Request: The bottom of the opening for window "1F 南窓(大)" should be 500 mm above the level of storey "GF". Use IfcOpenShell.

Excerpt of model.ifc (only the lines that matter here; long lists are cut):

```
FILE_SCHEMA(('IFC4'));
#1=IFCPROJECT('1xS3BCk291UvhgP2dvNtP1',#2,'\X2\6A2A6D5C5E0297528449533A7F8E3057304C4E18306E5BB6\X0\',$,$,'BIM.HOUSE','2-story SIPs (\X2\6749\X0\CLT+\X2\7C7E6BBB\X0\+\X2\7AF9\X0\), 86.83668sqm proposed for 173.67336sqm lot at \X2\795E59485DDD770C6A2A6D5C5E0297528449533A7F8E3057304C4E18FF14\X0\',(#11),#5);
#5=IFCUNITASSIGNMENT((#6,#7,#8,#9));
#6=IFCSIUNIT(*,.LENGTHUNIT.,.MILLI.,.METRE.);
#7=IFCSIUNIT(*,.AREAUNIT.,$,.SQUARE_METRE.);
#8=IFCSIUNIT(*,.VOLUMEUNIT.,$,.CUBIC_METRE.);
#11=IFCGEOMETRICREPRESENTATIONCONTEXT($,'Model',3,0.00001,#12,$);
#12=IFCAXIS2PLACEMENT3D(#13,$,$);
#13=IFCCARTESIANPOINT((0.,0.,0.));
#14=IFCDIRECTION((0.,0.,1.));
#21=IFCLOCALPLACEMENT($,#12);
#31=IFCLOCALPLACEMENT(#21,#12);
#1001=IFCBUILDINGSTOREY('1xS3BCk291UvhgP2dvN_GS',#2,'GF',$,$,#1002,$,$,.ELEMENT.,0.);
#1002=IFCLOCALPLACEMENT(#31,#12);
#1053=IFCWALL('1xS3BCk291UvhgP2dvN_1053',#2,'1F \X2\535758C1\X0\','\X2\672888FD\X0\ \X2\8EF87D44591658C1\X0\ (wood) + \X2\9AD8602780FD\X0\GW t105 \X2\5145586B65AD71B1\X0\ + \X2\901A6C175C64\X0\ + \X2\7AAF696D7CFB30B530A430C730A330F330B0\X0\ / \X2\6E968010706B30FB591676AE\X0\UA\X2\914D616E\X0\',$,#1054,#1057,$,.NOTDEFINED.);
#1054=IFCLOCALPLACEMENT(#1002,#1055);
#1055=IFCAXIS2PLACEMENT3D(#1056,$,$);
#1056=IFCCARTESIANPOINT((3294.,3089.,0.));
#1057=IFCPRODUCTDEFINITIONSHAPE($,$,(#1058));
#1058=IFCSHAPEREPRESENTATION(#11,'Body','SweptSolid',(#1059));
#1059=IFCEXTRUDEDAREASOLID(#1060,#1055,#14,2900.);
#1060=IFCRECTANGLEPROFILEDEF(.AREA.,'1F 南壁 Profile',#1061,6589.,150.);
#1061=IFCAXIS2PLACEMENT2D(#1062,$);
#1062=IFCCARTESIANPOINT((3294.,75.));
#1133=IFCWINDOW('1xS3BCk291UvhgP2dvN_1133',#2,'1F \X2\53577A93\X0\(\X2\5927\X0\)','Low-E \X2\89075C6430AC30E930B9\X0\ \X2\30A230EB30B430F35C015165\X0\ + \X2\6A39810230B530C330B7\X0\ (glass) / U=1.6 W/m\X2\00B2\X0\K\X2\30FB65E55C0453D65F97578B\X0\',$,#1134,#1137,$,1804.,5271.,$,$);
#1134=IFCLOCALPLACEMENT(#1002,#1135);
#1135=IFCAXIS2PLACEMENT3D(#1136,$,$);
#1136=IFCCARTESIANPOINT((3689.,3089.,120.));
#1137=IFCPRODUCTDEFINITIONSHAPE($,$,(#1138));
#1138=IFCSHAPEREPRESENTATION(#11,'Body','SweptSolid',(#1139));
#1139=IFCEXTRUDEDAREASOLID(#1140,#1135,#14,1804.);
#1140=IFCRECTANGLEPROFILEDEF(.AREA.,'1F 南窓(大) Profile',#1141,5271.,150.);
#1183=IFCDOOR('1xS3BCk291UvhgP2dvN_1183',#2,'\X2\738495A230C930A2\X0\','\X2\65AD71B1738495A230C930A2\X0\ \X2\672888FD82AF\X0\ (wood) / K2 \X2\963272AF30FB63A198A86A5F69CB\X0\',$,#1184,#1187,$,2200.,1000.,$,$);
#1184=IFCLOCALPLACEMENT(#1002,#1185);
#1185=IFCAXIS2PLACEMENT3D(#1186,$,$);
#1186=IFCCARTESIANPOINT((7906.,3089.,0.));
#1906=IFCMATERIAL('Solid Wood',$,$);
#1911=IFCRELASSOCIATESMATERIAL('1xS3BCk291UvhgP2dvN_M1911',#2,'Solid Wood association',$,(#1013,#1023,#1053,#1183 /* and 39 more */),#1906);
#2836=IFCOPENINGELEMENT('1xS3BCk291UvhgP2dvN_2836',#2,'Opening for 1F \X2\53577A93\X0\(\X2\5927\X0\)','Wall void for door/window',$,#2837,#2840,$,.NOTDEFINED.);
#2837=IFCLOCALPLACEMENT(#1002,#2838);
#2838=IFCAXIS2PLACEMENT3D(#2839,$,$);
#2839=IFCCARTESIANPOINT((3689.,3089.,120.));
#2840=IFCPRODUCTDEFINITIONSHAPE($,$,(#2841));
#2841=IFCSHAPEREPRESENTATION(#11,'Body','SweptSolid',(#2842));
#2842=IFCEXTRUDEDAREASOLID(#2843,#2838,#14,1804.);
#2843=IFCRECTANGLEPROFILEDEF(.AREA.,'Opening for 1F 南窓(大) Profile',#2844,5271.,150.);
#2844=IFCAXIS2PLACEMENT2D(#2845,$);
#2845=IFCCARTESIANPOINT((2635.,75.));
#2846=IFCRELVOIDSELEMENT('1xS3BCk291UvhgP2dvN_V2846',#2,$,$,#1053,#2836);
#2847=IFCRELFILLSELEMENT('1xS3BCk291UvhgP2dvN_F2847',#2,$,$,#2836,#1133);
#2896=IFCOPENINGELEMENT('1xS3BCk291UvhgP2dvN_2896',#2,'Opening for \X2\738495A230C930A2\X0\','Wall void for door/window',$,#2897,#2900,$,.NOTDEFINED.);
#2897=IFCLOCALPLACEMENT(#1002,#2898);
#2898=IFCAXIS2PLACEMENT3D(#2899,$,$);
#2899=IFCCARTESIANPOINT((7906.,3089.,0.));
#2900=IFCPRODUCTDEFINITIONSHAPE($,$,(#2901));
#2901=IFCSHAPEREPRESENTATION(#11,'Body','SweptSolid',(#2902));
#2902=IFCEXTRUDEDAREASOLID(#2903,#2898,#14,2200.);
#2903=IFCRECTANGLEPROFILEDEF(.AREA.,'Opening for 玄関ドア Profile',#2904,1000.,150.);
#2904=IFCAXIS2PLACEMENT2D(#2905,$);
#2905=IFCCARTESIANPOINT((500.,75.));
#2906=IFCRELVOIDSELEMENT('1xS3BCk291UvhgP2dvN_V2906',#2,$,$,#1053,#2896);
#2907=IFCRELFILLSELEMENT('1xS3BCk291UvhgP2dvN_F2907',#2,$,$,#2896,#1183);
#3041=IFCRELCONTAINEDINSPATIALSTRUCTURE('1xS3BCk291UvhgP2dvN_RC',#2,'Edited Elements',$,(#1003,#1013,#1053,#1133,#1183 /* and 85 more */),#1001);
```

```python
import numpy as np
import ifcopenshell
import ifcopenshell.api.geometry
import ifcopenshell.geom
import ifcopenshell.util.element
import ifcopenshell.util.placement
import ifcopenshell.util.shape
import ifcopenshell.util.unit

model = ifcopenshell.open("model.ifc")
unit_scale = ifcopenshell.util.unit.calculate_unit_scale(model)

window = model.by_id(1133)
opening = window.FillsVoids[0].RelatingOpeningElement
storey = ifcopenshell.util.element.get_container(window, ifc_class="IfcBuildingStorey")
level = ifcopenshell.util.placement.get_local_placement(storey.ObjectPlacement)[2, 3]

# The opening's origin need not be at the sill, so measure its lowest point.
shape = ifcopenshell.geom.create_shape(ifcopenshell.geom.settings(), opening)
bottom = ifcopenshell.util.shape.get_shape_bottom_elevation(shape, shape.geometry) / unit_scale
dz = level + 500.0 - bottom

shift = np.array([0.0, 0.0, dz])
# The window is not placed relative to its opening, so move both.
for product in (opening, window):
    matrix = ifcopenshell.util.placement.get_local_placement(product.ObjectPlacement)
    matrix[:3, 3] += shift
    ifcopenshell.api.geometry.edit_object_placement(model, product=product, matrix=matrix, is_si=False)

print(f"moved by {dz * unit_scale:+.3f} m")

model.write("model_rev.ifc")
```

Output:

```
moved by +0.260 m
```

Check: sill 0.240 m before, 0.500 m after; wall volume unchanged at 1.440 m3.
